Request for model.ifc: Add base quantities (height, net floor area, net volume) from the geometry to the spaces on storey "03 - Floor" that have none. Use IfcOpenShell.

First a look at what the model holds.

```python
import ifcopenshell
import ifcopenshell.util.element
import ifcopenshell.util.unit

model = ifcopenshell.open("model.ifc")
print(model.schema)
for unit_type in ("LENGTHUNIT", "AREAUNIT", "VOLUMEUNIT"):
    print(unit_type, ifcopenshell.util.unit.calculate_unit_scale(model, unit_type))
storey = next(s for s in model.by_type("IfcBuildingStorey") if s.Name == "03 - Floor")
spaces = [e for e in ifcopenshell.util.element.get_decomposition(storey) if e.is_a("IfcSpace")]
for e in sorted(spaces, key=lambda e: e.id()):
    print(e.id(), e.is_a(), e.Name, list(ifcopenshell.util.element.get_psets(e, qtos_only=True)), sep=" | ")
```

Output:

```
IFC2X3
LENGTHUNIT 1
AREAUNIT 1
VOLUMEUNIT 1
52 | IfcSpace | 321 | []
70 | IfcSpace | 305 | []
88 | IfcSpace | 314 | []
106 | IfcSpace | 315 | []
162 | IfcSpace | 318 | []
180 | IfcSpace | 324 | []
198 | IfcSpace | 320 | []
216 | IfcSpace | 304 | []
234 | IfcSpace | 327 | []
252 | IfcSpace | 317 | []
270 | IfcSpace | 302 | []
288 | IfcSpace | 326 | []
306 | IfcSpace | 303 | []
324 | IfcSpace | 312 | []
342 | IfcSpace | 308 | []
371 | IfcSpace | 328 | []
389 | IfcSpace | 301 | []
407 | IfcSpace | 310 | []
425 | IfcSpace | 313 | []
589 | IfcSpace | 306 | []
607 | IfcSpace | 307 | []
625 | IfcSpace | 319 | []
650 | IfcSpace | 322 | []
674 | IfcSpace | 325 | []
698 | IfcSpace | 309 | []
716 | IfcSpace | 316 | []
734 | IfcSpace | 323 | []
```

```python
import ifcopenshell
import ifcopenshell.api.pset
import ifcopenshell.geom
import ifcopenshell.util.element
import ifcopenshell.util.shape
import ifcopenshell.util.unit

model = ifcopenshell.open("model.ifc")
unit_scale = ifcopenshell.util.unit.calculate_unit_scale(model)
area_scale = ifcopenshell.util.unit.calculate_unit_scale(model, "AREAUNIT")
volume_scale = ifcopenshell.util.unit.calculate_unit_scale(model, "VOLUMEUNIT")
settings = ifcopenshell.geom.settings()

storey = next(s for s in model.by_type("IfcBuildingStorey") if s.Name == "03 - Floor")
spaces = [e for e in ifcopenshell.util.element.get_decomposition(storey) if e.is_a("IfcSpace")]

for e in sorted(spaces, key=lambda e: e.id()):
    if ifcopenshell.util.element.get_psets(e, qtos_only=True, should_inherit=False):
        continue
    # Geometry comes back in metres, in the element's own axes.
    shape = ifcopenshell.geom.create_shape(settings, e)
    values = {
        "Height": ifcopenshell.util.shape.get_z(shape.geometry) / unit_scale,
        "NetFloorArea": ifcopenshell.util.shape.get_footprint_area(shape.geometry) / area_scale,
        "NetVolume": ifcopenshell.util.shape.get_volume(shape.geometry) / volume_scale,
    }
    qto = ifcopenshell.api.pset.add_qto(model, product=e, name="BaseQuantities")
    ifcopenshell.api.pset.edit_qto(model, qto=qto, properties=values)
    print(e.id(), {k: round(v, 3) for k, v in values.items()})

model.write("model-out.ifc")
```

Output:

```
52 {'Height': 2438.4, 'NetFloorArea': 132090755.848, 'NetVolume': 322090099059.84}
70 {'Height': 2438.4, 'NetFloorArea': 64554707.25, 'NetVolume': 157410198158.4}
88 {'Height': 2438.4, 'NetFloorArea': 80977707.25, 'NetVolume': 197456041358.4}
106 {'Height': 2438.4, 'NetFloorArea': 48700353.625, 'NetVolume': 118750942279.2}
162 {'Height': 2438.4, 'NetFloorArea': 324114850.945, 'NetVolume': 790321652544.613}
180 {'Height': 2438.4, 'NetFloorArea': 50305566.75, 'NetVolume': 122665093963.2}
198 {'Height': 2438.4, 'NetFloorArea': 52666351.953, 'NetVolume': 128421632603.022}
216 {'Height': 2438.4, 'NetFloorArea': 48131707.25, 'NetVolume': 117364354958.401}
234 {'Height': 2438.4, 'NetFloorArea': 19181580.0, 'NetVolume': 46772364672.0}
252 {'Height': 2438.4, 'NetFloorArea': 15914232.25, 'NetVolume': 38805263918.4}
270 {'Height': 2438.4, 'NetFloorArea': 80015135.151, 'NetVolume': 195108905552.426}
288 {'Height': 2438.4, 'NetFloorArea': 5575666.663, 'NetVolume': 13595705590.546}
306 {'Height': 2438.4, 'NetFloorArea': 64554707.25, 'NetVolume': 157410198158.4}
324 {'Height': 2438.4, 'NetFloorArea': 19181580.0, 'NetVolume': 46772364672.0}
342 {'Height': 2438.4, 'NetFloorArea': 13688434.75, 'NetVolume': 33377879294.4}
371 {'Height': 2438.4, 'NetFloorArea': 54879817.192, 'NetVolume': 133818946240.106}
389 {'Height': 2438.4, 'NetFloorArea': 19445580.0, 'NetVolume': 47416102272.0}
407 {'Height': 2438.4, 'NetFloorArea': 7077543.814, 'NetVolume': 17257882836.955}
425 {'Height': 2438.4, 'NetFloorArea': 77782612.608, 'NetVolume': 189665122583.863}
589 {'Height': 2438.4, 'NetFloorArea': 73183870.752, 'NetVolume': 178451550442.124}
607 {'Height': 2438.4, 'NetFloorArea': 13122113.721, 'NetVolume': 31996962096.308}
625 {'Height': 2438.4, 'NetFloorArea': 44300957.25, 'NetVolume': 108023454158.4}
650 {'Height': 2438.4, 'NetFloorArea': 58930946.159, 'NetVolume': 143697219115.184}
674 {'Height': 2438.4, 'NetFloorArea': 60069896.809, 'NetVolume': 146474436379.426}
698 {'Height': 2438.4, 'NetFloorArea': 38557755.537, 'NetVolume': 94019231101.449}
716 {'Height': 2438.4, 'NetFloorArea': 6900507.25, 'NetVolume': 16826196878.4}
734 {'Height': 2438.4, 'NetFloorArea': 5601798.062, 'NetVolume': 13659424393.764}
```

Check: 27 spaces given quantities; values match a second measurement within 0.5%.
